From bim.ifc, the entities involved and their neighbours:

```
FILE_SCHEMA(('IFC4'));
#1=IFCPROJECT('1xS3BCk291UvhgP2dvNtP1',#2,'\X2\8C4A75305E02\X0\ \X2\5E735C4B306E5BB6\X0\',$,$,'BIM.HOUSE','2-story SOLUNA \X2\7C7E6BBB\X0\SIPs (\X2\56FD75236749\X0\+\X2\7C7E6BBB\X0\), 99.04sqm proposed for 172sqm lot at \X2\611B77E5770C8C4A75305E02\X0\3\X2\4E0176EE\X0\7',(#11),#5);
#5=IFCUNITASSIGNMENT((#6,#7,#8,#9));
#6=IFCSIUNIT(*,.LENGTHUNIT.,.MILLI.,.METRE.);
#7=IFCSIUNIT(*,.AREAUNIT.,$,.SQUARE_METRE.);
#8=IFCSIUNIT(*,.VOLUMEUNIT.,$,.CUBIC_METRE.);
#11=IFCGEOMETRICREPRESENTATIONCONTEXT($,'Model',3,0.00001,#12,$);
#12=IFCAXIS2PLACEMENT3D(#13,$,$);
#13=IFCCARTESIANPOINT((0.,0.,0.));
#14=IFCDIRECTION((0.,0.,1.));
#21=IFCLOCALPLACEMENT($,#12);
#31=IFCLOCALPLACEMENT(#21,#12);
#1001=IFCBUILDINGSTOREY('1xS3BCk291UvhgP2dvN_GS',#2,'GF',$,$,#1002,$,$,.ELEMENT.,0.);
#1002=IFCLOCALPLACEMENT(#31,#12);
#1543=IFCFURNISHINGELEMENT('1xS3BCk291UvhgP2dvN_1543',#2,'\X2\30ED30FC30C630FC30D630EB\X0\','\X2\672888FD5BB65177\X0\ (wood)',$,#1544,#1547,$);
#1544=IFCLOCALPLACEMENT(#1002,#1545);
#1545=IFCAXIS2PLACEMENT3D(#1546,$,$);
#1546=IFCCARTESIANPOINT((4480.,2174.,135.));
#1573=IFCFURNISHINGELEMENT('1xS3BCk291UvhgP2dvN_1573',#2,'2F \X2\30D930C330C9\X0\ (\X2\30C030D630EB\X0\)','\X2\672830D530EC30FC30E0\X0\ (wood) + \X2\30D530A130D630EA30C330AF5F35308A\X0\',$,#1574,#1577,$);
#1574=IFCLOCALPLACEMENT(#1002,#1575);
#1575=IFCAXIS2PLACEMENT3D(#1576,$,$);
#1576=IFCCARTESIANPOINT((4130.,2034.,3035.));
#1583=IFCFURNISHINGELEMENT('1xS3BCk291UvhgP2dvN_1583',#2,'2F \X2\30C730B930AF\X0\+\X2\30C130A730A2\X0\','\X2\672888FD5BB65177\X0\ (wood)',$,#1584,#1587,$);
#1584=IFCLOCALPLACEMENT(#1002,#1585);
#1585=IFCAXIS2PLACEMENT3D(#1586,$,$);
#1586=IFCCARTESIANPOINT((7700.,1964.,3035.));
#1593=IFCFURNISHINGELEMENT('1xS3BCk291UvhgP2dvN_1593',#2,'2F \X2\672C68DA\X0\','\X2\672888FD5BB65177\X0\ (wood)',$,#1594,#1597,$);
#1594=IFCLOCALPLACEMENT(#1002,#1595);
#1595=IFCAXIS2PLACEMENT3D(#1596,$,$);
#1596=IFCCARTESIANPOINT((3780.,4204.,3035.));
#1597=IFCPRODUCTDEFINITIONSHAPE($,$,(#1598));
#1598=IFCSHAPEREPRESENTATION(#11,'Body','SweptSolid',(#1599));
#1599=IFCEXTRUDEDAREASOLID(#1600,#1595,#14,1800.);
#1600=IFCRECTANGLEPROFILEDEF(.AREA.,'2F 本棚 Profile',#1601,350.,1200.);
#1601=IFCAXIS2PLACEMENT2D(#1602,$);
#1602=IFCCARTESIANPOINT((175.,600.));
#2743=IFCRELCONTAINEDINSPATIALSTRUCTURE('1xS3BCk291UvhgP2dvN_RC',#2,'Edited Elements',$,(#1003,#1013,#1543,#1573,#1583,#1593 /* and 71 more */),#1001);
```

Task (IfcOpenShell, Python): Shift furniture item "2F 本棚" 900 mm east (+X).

```python
import ifcopenshell
import ifcopenshell.api.geometry
import ifcopenshell.util.placement
import ifcopenshell.util.unit

model = ifcopenshell.open("bim.ifc")
unit_scale = ifcopenshell.util.unit.calculate_unit_scale(model)

item = model.by_guid("1xS3BCk291UvhgP2dvN_1593")
matrix = ifcopenshell.util.placement.get_local_placement(item.ObjectPlacement)
matrix[0, 3] += 0.9 / unit_scale
ifcopenshell.api.geometry.edit_object_placement(model, product=item, matrix=matrix, is_si=False)

print(ifcopenshell.util.placement.get_local_placement(item.ObjectPlacement).round(3) + 0.0)

model.write("bim-out.ifc")
```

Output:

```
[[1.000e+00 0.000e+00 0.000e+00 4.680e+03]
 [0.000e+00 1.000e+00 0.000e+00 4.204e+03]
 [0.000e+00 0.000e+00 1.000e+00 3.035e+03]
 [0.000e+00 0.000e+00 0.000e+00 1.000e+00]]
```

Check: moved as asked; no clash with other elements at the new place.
